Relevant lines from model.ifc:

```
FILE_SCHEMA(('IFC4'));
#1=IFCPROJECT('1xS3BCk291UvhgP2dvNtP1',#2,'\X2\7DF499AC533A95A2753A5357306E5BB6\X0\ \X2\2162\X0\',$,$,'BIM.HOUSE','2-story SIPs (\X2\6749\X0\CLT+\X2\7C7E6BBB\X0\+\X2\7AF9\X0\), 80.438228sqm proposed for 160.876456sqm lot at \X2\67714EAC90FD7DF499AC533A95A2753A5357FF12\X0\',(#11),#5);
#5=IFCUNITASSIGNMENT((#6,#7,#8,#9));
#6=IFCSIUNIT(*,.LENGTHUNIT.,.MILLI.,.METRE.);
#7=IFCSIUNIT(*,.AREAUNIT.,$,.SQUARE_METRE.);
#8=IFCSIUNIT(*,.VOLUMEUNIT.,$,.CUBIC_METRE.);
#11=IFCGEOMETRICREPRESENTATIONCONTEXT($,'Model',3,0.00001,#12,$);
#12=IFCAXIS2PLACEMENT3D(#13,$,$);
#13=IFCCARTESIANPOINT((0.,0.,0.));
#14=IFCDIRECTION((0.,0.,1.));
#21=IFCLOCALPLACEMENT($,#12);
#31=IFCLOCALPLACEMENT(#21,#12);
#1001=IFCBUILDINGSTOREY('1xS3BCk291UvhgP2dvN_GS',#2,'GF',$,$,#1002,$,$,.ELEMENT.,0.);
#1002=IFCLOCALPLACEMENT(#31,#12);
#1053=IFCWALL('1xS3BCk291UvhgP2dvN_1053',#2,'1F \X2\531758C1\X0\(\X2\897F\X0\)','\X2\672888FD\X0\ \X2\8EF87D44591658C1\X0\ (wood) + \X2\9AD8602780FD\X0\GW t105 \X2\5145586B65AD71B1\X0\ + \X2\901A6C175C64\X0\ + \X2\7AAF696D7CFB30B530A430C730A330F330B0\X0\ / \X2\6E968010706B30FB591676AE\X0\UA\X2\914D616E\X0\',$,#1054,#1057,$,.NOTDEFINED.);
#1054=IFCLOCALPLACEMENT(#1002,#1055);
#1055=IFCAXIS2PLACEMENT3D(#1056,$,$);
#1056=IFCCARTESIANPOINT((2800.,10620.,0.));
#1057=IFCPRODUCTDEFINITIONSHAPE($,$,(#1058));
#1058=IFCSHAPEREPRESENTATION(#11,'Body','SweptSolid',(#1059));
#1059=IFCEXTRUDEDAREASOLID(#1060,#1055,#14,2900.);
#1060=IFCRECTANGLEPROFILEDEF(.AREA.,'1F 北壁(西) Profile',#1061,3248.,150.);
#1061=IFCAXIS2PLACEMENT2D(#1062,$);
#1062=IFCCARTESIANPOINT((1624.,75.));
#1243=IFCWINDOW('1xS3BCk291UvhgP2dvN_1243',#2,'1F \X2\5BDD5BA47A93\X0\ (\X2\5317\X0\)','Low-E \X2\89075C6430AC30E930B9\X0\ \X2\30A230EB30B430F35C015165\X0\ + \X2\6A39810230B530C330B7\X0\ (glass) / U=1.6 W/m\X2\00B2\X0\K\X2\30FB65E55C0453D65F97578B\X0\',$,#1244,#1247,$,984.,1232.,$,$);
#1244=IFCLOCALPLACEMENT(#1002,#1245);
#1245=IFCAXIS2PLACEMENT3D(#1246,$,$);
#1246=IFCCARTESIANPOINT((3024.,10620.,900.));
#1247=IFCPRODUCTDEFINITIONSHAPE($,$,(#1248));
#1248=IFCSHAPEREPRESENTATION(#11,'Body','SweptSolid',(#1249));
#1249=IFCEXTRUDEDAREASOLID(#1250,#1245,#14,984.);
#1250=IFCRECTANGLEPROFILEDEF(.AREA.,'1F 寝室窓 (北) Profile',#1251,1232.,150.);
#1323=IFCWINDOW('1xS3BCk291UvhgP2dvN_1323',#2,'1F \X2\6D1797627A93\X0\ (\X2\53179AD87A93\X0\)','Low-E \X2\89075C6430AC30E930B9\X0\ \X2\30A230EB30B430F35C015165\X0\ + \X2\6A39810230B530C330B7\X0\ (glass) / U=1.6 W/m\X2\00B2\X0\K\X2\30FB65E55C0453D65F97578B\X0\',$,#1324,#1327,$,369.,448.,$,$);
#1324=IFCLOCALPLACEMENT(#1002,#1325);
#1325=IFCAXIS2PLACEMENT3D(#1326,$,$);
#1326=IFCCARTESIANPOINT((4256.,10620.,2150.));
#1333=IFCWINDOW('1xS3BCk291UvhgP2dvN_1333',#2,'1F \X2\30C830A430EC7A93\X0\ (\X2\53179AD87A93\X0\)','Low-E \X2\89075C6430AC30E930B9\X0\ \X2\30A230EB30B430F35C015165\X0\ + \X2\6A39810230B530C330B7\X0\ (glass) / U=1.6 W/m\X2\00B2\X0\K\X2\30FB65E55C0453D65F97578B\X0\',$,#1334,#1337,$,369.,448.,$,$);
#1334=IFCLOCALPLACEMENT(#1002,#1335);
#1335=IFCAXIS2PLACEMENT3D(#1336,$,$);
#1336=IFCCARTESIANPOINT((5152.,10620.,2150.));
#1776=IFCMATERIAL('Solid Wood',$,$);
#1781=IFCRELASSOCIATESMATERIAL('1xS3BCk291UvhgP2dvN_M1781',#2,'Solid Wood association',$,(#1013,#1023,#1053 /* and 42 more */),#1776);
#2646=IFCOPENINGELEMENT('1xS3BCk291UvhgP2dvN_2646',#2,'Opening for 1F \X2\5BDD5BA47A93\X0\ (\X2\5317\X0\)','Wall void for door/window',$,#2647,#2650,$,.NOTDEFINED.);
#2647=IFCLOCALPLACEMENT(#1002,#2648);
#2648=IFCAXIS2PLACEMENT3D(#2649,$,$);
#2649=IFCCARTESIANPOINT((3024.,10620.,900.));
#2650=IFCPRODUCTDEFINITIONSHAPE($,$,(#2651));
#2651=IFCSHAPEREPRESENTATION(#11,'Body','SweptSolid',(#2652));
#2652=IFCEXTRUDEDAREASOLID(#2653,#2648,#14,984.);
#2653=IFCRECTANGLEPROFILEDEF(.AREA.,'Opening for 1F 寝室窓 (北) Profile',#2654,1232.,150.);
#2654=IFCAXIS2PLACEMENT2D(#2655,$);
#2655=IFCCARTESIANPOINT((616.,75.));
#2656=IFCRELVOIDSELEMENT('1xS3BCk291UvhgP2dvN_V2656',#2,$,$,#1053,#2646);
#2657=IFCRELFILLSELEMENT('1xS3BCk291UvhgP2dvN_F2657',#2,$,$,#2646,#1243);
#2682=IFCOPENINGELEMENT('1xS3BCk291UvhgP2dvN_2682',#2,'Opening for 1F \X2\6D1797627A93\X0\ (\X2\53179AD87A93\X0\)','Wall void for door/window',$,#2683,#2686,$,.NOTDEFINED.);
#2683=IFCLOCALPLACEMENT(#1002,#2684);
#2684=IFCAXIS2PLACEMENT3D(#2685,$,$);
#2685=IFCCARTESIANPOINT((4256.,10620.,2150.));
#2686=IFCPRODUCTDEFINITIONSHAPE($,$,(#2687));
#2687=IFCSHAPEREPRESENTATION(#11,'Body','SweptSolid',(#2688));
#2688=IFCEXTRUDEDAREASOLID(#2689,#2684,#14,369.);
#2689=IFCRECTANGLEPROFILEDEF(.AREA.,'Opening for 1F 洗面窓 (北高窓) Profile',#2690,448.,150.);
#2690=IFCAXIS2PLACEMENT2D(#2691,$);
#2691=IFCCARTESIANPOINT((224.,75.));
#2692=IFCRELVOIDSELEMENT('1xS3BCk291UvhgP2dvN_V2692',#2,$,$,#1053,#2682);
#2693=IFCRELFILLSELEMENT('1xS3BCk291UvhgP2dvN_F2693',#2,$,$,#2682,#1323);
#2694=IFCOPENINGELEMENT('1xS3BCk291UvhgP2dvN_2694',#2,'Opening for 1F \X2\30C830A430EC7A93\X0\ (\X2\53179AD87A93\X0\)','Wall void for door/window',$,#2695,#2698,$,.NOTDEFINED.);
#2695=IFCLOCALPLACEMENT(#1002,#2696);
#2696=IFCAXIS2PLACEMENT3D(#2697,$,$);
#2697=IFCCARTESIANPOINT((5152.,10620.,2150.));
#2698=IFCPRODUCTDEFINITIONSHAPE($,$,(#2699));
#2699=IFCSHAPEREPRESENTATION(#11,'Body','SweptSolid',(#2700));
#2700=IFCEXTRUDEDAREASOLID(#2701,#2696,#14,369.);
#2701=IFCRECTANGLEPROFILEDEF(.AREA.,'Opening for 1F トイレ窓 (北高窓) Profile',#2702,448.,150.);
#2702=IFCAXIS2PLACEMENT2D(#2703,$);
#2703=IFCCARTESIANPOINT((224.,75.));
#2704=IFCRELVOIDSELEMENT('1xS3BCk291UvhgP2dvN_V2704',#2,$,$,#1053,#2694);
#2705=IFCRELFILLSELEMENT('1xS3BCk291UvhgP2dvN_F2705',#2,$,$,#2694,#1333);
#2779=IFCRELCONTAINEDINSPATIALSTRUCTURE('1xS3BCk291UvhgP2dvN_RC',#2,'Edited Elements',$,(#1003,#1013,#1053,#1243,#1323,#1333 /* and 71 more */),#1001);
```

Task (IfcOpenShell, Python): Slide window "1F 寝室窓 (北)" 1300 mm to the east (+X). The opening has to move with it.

```python
import ifcopenshell
import ifcopenshell.api.geometry
import ifcopenshell.util.placement
import ifcopenshell.util.unit

model = ifcopenshell.open("model.ifc")
unit_scale = ifcopenshell.util.unit.calculate_unit_scale(model)

window = model.by_guid("1xS3BCk291UvhgP2dvN_1243")
opening = window.FillsVoids[0].RelatingOpeningElement
wall = opening.VoidsElements[0].RelatingBuildingElement

wall_matrix = ifcopenshell.util.placement.get_local_placement(wall.ObjectPlacement)
shift = wall_matrix[:3, 0] * 1.3 / unit_scale
before = ifcopenshell.util.placement.get_local_placement(window.ObjectPlacement)[:3, 3].copy()

# The window is not placed relative to its opening, so move both.
for product in (opening, window):
    matrix = ifcopenshell.util.placement.get_local_placement(product.ObjectPlacement)
    matrix[:3, 3] += shift
    ifcopenshell.api.geometry.edit_object_placement(model, product=product, matrix=matrix, is_si=False)

after = ifcopenshell.util.placement.get_local_placement(window.ObjectPlacement)[:3, 3]
print("window moved by", (after - before).round(3) + 0.0)

model.write("model-out.ifc")
```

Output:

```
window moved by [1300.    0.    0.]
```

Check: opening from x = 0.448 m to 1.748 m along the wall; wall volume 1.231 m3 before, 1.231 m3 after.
